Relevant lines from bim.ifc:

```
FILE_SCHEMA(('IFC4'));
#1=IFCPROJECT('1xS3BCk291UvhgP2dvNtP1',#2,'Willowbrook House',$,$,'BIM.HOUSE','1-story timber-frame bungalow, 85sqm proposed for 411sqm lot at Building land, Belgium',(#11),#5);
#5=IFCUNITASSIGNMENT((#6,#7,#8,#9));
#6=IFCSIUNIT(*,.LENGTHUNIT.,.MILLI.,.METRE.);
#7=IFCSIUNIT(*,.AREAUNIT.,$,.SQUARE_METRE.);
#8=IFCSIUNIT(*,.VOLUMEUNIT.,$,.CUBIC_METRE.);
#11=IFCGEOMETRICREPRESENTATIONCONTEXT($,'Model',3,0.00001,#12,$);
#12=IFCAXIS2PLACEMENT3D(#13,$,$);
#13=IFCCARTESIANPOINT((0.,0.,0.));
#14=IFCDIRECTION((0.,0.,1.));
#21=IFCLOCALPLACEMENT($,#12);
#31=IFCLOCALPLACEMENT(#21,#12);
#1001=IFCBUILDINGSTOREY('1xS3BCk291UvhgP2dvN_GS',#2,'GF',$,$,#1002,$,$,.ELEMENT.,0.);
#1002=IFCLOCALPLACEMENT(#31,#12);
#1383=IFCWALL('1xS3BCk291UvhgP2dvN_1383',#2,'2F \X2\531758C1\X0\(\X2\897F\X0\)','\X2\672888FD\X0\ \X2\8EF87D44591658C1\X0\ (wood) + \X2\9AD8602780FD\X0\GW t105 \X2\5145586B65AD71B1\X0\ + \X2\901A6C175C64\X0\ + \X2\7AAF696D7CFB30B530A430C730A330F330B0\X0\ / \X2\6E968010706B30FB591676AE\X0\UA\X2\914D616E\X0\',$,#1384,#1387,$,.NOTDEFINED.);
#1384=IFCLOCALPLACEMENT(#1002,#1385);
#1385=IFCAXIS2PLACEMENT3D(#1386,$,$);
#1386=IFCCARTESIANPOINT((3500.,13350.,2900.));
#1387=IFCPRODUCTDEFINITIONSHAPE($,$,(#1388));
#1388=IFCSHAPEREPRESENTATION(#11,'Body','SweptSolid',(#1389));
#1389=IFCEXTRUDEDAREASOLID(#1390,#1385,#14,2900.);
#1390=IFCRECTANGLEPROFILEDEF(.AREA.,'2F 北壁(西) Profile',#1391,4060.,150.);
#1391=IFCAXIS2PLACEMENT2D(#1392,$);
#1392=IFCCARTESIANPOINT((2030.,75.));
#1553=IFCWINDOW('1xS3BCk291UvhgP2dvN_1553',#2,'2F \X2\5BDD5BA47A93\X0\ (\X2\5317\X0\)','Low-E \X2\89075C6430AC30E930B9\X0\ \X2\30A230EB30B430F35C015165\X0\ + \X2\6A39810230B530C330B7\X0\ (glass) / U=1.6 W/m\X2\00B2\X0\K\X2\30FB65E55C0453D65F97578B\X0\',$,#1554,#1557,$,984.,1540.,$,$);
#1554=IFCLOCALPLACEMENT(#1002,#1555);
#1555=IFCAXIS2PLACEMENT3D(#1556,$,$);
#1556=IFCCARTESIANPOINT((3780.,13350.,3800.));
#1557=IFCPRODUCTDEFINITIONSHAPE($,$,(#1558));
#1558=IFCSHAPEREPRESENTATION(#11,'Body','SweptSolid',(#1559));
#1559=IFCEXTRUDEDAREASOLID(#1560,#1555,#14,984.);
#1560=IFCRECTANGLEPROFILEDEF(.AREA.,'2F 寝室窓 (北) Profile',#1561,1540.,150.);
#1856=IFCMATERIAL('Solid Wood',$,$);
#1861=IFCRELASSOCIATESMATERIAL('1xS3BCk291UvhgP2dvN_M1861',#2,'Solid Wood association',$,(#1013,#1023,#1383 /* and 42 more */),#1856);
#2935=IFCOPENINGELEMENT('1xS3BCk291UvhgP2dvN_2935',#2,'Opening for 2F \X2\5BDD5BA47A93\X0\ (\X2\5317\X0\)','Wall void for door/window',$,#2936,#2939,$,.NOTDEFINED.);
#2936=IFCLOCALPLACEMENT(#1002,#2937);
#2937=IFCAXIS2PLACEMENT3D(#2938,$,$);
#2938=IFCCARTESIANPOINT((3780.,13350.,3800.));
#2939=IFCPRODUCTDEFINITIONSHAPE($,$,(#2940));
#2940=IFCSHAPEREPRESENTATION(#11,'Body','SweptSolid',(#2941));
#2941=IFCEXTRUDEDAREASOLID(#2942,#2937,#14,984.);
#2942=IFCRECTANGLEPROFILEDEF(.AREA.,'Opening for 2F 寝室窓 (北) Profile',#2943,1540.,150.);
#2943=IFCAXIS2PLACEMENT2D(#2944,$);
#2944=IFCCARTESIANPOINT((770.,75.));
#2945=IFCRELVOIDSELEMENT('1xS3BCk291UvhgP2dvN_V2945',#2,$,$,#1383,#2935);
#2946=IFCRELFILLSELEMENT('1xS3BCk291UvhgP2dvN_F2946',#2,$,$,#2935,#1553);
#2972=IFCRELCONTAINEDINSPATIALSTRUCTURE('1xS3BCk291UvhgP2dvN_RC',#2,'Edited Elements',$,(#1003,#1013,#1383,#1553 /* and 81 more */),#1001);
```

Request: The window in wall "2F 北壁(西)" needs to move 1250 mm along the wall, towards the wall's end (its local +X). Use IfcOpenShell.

```python
import ifcopenshell
import ifcopenshell.api.geometry
import ifcopenshell.util.placement

model = ifcopenshell.open("bim.ifc")

window = model.by_guid("1xS3BCk291UvhgP2dvN_1553")
opening = window.FillsVoids[0].RelatingOpeningElement
wall = opening.VoidsElements[0].RelatingBuildingElement

wall_matrix = ifcopenshell.util.placement.get_local_placement(wall.ObjectPlacement)
shift = wall_matrix[:3, 0] * 1250.0
before = ifcopenshell.util.placement.get_local_placement(window.ObjectPlacement)[:3, 3].copy()

# The window is not placed relative to its opening, so move both.
for product in (opening, window):
    matrix = ifcopenshell.util.placement.get_local_placement(product.ObjectPlacement)
    matrix[:3, 3] += shift
    ifcopenshell.api.geometry.edit_object_placement(model, product=product, matrix=matrix, is_si=False)

after = ifcopenshell.util.placement.get_local_placement(window.ObjectPlacement)[:3, 3]
print("window moved by", (after - before).round(3) + 0.0)

model.write("bim_v2.ifc")
```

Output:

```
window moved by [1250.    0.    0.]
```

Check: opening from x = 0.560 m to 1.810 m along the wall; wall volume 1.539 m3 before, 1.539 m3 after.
